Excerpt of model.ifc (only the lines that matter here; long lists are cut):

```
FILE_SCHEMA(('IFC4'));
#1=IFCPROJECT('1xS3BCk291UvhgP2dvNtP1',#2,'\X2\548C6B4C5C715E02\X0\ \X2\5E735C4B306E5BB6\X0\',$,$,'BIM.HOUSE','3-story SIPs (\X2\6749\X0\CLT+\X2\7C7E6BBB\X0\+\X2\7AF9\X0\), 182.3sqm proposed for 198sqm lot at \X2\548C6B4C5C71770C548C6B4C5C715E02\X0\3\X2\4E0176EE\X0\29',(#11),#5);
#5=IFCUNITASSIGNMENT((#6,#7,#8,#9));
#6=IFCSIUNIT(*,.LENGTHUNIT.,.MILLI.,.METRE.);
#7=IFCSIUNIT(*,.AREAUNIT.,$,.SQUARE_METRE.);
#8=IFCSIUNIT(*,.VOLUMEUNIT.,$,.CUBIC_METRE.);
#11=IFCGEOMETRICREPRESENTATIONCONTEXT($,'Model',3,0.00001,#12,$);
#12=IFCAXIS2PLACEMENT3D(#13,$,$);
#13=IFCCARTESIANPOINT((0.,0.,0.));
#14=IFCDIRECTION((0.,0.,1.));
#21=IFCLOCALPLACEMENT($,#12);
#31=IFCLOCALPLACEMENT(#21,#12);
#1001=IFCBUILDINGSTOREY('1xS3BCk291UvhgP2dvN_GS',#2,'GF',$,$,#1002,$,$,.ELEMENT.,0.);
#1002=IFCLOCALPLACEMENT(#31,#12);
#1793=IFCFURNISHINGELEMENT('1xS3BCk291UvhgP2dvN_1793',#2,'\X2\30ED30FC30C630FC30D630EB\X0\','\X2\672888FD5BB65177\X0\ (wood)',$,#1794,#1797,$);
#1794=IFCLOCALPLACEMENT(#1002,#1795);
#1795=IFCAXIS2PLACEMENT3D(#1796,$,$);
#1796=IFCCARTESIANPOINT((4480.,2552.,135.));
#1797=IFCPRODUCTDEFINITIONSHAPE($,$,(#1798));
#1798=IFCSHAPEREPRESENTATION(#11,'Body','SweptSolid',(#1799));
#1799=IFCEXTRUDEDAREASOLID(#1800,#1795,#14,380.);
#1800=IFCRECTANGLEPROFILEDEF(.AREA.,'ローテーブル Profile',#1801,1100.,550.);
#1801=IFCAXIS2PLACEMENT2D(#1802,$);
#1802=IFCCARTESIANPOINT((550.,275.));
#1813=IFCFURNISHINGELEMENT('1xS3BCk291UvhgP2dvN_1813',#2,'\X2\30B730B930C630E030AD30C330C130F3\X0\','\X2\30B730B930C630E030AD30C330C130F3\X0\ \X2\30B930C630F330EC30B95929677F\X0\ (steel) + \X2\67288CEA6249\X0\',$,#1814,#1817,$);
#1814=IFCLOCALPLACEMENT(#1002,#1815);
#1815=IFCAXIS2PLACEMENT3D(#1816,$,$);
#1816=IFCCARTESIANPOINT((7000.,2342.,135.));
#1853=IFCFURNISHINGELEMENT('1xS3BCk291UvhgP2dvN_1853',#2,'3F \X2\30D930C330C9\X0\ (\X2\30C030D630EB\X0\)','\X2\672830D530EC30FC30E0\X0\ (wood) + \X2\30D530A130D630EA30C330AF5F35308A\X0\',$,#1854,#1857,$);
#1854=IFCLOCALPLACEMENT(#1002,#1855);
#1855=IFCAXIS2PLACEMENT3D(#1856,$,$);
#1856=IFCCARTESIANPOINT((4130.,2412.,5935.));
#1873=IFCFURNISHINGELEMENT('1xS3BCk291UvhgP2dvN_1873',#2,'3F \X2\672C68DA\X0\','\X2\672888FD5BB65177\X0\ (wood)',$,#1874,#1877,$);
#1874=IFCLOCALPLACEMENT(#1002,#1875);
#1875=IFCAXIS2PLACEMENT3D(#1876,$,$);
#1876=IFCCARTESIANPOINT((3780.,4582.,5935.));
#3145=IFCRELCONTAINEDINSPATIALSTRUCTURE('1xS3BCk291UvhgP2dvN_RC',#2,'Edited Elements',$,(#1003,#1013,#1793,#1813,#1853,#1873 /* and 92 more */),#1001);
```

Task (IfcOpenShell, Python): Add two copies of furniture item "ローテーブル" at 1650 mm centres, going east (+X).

```python
import numpy as np
import ifcopenshell
import ifcopenshell.api.geometry
import ifcopenshell.api.root
import ifcopenshell.util.element
import ifcopenshell.util.placement
import ifcopenshell.util.unit

model = ifcopenshell.open("model.ifc")
unit_scale = ifcopenshell.util.unit.calculate_unit_scale(model)


def reuse_history(source, copy):
    """copy_class also copies each property set's owner history, people and application; keep the originals."""
    for rel in copy.IsDefinedBy:
        if rel.is_a("IfcRelDefinesByProperties") and (history := rel.RelatingPropertyDefinition.OwnerHistory):
            rel.RelatingPropertyDefinition.OwnerHistory = source.OwnerHistory
            ifcopenshell.util.element.remove_deep2(model, history)


source = model.by_id(1793)
base = ifcopenshell.util.placement.get_local_placement(source.ObjectPlacement)
step = np.array([1.0, 0.0, 0.0]) * 1.65 / unit_scale

for i in range(1, 3):
    copy = ifcopenshell.api.root.copy_class(model, product=source)
    copy.Representation = ifcopenshell.util.element.copy_deep(
        model, source.Representation, exclude=["IfcGeometricRepresentationContext", "IfcRepresentationMap"]
    )
    reuse_history(source, copy)
    matrix = base.copy()
    matrix[:3, 3] += i * step
    print("added at", matrix[:3, 3].round(3) + 0.0)
    ifcopenshell.api.geometry.edit_object_placement(model, product=copy, matrix=matrix, is_si=False)

model.write("model_rev.ifc")
```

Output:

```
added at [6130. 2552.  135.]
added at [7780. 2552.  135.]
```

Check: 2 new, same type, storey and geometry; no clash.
